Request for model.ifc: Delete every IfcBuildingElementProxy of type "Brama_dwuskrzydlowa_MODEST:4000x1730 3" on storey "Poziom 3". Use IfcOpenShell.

First a look at what the model holds.

```python
import ifcopenshell
import ifcopenshell.util.element

model = ifcopenshell.open("model.ifc")
print(model.schema)
storey = next(s for s in model.by_type("IfcBuildingStorey") if s.Name == "Poziom 3")
proxies = [e for e in ifcopenshell.util.element.get_decomposition(storey) if e.is_a("IfcBuildingElementProxy")]
seen = {}
for e in proxies:
    element_type = ifcopenshell.util.element.get_type(e)
    name = element_type.Name if element_type not in (None, e) else None
    seen[name] = seen.get(name, 0) + 1
for name, count in sorted(seen.items(), key=str):
    print(count, "x", name)
```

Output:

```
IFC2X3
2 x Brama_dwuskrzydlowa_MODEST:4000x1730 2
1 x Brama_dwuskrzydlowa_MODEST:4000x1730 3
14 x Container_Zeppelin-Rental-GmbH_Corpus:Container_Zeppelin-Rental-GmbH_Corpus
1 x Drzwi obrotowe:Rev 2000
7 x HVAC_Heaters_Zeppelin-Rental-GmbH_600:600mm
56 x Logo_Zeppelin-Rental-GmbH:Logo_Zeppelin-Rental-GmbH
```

```python
import ifcopenshell
import ifcopenshell.api.root
import ifcopenshell.util.element

model = ifcopenshell.open("model.ifc")

storey = next(s for s in model.by_type("IfcBuildingStorey") if s.Name == "Poziom 3")
proxies = [e for e in ifcopenshell.util.element.get_decomposition(storey) if e.is_a("IfcBuildingElementProxy")]
targets = [e for e in proxies if (t := ifcopenshell.util.element.get_type(e)) not in (None, e) and t.Name == "Brama_dwuskrzydlowa_MODEST:4000x1730 3"]

for e in targets:
    ifcopenshell.api.root.remove_product(model, product=e)
print(len(targets), "removed")

model.write("model-out.ifc")
```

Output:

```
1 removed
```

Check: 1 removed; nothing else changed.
